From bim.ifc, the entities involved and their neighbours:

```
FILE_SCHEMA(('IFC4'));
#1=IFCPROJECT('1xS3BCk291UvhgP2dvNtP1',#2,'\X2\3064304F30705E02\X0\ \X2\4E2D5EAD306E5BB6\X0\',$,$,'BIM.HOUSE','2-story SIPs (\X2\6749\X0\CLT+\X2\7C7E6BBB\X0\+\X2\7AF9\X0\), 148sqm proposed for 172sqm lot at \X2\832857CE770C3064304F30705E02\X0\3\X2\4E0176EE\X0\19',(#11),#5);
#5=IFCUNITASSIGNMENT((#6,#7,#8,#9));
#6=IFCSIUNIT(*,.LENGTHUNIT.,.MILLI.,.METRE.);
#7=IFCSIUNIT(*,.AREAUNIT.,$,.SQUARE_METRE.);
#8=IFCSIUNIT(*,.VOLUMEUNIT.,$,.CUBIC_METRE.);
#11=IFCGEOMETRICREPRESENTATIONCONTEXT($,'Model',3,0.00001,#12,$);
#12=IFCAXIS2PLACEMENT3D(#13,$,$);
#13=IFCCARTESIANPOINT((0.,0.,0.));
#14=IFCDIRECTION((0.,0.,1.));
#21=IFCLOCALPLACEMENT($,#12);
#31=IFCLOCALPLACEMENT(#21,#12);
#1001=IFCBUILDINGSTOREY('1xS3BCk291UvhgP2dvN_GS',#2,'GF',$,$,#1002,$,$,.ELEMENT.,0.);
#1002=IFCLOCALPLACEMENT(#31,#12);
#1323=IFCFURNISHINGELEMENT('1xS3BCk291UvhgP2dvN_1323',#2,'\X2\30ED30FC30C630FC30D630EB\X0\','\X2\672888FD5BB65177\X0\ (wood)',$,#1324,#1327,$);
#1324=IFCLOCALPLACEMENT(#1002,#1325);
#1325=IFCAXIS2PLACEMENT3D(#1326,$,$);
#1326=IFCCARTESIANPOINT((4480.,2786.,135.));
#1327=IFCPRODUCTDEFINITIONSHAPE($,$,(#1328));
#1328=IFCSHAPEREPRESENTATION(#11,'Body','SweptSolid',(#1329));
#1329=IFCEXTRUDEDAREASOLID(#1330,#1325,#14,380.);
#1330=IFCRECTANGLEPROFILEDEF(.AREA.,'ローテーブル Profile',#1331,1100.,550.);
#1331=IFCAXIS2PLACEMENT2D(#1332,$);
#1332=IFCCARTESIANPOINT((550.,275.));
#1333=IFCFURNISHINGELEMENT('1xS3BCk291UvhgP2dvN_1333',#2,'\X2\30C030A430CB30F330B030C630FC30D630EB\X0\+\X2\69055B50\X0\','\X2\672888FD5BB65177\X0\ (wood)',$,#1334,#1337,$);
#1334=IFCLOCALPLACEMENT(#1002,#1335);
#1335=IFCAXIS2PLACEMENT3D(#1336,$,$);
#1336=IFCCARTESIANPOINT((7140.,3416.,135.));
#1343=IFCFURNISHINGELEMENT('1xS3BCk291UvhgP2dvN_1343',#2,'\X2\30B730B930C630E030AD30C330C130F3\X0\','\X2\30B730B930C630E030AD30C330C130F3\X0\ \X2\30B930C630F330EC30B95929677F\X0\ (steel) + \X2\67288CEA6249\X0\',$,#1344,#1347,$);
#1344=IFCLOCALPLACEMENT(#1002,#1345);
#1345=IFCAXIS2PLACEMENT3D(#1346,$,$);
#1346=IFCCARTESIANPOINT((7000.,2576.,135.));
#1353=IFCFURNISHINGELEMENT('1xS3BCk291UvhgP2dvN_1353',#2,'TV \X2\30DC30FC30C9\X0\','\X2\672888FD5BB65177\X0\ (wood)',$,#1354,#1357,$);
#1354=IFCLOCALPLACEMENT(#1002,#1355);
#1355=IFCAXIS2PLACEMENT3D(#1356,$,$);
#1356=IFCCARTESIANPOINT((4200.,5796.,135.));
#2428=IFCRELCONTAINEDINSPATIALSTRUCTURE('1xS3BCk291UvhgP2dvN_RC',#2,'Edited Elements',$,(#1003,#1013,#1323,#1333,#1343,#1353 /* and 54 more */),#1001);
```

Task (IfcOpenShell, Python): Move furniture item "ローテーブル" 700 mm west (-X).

```python
import ifcopenshell
import ifcopenshell.api.geometry
import ifcopenshell.util.placement

model = ifcopenshell.open("bim.ifc")

item = model.by_guid("1xS3BCk291UvhgP2dvN_1323")
matrix = ifcopenshell.util.placement.get_local_placement(item.ObjectPlacement)
matrix[0, 3] -= 700.0
ifcopenshell.api.geometry.edit_object_placement(model, product=item, matrix=matrix, is_si=False)

print(ifcopenshell.util.placement.get_local_placement(item.ObjectPlacement).round(3) + 0.0)

model.write("bim-out.ifc")
```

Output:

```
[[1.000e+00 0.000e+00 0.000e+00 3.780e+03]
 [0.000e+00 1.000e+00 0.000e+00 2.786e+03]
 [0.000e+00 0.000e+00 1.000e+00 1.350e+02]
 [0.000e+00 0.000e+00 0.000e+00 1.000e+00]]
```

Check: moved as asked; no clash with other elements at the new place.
